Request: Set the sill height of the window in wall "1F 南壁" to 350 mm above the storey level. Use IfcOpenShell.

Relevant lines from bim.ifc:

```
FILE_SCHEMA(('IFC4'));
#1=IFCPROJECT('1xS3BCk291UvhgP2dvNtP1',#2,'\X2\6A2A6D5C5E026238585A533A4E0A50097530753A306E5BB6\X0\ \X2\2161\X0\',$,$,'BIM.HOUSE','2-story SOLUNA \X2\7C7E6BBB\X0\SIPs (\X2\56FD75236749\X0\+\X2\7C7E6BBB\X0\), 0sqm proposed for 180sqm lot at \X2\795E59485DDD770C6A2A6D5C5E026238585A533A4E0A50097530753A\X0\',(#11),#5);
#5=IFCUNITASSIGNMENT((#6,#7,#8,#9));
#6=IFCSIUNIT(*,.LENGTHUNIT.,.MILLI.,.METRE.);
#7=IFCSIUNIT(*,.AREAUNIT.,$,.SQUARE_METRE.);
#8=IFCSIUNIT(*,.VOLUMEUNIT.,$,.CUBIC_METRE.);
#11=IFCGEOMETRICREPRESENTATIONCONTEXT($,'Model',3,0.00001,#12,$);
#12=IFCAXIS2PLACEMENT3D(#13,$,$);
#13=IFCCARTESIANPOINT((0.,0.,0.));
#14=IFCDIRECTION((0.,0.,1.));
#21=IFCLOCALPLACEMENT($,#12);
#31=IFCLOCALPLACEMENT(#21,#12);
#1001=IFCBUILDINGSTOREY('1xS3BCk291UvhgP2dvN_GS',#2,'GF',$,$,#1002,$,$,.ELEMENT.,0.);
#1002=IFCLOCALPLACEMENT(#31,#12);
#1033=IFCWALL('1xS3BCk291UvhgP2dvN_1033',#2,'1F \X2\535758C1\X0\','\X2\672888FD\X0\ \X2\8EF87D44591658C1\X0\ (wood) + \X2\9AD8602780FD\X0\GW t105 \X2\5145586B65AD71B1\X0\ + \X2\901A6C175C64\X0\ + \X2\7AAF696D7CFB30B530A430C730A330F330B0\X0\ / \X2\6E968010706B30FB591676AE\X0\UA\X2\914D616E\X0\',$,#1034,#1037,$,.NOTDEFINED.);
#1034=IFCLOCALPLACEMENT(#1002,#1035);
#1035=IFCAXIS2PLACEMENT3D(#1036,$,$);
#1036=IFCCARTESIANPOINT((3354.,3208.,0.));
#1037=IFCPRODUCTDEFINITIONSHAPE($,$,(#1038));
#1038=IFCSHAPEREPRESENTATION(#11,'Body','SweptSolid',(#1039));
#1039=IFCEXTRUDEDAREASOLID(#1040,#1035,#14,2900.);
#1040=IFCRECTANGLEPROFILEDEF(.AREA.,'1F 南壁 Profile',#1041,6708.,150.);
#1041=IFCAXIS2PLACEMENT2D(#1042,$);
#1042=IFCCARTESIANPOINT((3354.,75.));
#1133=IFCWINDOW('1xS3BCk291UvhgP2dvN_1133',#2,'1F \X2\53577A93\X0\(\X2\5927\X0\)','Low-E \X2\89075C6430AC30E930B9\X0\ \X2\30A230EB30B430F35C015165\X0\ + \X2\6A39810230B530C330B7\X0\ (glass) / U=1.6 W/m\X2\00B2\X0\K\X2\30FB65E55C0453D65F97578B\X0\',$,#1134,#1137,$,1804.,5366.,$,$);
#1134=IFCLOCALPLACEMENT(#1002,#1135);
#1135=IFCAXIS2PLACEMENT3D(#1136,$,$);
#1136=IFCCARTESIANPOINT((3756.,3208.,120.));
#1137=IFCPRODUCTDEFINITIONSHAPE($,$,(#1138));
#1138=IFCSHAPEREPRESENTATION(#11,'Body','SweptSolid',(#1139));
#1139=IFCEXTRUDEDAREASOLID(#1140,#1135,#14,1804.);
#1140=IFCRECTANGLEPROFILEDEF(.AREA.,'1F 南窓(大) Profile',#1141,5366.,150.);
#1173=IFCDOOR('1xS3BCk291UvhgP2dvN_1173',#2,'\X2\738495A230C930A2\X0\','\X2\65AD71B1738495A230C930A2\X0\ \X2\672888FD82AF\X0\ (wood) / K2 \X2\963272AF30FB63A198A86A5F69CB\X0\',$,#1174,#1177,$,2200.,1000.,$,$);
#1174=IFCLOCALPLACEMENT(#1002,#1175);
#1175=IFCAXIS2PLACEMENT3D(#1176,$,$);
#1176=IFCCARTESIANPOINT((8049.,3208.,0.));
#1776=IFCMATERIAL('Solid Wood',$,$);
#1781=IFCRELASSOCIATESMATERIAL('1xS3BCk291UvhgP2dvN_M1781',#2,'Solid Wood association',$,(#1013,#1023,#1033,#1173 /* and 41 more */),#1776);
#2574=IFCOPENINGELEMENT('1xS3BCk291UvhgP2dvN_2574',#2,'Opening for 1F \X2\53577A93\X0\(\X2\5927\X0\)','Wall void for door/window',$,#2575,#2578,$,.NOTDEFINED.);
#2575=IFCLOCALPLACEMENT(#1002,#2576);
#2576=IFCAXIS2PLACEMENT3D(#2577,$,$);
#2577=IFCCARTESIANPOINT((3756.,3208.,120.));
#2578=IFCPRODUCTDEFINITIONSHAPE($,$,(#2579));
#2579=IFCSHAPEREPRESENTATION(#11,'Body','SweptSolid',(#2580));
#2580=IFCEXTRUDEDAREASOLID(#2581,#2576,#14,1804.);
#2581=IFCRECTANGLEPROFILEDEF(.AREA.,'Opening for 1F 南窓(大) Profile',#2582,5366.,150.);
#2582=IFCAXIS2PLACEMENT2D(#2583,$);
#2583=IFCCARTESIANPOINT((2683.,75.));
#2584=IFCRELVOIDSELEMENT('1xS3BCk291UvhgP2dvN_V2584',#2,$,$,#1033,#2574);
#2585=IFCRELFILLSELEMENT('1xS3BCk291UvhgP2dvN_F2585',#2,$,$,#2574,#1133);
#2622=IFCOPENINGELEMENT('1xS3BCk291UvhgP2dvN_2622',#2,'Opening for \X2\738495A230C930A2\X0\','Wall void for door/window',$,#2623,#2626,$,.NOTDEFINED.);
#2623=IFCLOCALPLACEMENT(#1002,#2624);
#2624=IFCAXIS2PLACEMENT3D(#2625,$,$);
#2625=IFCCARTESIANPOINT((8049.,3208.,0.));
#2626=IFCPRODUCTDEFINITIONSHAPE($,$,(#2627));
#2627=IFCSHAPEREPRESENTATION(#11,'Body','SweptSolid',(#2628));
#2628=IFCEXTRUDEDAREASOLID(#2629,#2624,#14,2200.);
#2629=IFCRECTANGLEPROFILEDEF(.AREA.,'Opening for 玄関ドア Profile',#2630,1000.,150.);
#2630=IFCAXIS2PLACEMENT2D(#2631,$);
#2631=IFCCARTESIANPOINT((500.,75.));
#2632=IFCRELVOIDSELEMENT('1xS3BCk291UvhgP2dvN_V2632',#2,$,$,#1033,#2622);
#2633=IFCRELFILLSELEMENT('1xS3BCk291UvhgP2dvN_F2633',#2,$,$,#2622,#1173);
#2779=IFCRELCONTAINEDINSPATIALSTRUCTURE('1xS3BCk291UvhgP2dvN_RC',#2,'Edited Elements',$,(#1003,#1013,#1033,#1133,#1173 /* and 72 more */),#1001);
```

```python
import numpy as np
import ifcopenshell
import ifcopenshell.api.geometry
import ifcopenshell.geom
import ifcopenshell.util.element
import ifcopenshell.util.placement
import ifcopenshell.util.shape
import ifcopenshell.util.unit

model = ifcopenshell.open("bim.ifc")
unit_scale = ifcopenshell.util.unit.calculate_unit_scale(model)

window = model.by_id(1133)
opening = window.FillsVoids[0].RelatingOpeningElement
storey = ifcopenshell.util.element.get_container(window, ifc_class="IfcBuildingStorey")
level = ifcopenshell.util.placement.get_local_placement(storey.ObjectPlacement)[2, 3]

# The opening's origin need not be at the sill, so measure its lowest point.
shape = ifcopenshell.geom.create_shape(ifcopenshell.geom.settings(), opening)
bottom = ifcopenshell.util.shape.get_shape_bottom_elevation(shape, shape.geometry) / unit_scale
dz = level + 0.35 / unit_scale - bottom

shift = np.array([0.0, 0.0, dz])
# The window is not placed relative to its opening, so move both.
for product in (opening, window):
    matrix = ifcopenshell.util.placement.get_local_placement(product.ObjectPlacement)
    matrix[:3, 3] += shift
    ifcopenshell.api.geometry.edit_object_placement(model, product=product, matrix=matrix, is_si=False)

print(f"moved by {dz * unit_scale:+.3f} m")

model.write("bim-out.ifc")
```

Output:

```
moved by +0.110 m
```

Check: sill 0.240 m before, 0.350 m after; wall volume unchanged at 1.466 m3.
